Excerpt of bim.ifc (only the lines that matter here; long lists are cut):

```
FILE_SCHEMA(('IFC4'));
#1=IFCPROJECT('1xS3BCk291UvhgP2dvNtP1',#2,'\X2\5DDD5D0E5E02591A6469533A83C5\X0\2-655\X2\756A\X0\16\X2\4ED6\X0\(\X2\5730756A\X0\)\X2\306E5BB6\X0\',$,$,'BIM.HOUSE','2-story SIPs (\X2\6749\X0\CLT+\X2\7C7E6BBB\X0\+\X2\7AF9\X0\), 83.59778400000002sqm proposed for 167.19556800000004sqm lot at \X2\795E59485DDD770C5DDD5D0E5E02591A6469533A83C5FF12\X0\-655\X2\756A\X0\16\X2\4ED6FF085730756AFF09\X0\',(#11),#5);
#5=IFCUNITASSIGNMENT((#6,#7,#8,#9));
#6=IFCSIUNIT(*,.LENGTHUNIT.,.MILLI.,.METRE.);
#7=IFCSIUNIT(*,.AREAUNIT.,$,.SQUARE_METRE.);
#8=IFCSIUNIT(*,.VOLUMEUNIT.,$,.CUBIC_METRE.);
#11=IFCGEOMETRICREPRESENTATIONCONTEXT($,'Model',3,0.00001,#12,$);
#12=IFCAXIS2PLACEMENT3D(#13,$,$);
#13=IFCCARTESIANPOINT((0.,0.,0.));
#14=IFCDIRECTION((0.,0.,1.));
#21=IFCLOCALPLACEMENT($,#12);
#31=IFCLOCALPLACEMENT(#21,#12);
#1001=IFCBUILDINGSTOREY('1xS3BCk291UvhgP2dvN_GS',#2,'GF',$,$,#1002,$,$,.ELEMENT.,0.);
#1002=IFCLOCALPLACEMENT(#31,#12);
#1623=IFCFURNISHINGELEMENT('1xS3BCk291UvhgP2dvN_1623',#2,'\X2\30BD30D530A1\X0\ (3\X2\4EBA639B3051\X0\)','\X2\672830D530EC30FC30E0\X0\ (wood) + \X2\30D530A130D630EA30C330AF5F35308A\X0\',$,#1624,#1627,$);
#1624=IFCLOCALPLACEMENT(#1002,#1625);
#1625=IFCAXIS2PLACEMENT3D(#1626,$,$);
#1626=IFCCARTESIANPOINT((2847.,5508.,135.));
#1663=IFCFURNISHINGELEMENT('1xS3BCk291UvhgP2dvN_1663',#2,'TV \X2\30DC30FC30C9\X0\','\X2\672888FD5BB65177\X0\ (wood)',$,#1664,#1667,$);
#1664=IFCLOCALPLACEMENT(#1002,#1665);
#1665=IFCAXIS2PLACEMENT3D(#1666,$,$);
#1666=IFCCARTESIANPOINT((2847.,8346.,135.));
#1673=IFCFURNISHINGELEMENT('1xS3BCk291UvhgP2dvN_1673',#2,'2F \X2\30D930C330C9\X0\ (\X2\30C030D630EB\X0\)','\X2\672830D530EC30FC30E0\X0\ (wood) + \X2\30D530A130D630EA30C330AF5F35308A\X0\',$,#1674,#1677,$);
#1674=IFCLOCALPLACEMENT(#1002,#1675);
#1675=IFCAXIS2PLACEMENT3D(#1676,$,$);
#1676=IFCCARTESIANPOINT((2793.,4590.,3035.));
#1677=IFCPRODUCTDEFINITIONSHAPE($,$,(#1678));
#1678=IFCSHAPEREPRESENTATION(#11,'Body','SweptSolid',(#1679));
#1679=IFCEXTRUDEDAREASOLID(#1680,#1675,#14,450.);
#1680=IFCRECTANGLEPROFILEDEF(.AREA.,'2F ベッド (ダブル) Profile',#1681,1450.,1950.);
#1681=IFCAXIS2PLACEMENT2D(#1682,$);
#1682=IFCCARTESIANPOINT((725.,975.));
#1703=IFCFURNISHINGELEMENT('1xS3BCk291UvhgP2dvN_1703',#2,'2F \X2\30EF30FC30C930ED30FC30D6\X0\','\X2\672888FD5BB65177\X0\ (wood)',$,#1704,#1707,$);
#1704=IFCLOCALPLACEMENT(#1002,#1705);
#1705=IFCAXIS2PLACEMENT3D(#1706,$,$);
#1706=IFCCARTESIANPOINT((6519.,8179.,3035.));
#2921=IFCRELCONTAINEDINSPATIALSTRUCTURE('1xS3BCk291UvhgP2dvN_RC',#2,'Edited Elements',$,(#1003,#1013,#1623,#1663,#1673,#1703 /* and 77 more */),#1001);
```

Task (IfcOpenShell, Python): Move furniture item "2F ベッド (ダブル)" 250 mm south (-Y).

```python
import ifcopenshell
import ifcopenshell.api.geometry
import ifcopenshell.util.placement

model = ifcopenshell.open("bim.ifc")

item = model.by_id(1673)
matrix = ifcopenshell.util.placement.get_local_placement(item.ObjectPlacement)
matrix[1, 3] -= 250.0
ifcopenshell.api.geometry.edit_object_placement(model, product=item, matrix=matrix, is_si=False)

print(ifcopenshell.util.placement.get_local_placement(item.ObjectPlacement).round(3) + 0.0)

model.write("bim_rev.ifc")
```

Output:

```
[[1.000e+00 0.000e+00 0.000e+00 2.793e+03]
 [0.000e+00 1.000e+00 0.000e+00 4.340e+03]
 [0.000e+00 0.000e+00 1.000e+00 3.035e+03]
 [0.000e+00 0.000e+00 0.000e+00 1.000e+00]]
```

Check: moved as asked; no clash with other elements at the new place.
